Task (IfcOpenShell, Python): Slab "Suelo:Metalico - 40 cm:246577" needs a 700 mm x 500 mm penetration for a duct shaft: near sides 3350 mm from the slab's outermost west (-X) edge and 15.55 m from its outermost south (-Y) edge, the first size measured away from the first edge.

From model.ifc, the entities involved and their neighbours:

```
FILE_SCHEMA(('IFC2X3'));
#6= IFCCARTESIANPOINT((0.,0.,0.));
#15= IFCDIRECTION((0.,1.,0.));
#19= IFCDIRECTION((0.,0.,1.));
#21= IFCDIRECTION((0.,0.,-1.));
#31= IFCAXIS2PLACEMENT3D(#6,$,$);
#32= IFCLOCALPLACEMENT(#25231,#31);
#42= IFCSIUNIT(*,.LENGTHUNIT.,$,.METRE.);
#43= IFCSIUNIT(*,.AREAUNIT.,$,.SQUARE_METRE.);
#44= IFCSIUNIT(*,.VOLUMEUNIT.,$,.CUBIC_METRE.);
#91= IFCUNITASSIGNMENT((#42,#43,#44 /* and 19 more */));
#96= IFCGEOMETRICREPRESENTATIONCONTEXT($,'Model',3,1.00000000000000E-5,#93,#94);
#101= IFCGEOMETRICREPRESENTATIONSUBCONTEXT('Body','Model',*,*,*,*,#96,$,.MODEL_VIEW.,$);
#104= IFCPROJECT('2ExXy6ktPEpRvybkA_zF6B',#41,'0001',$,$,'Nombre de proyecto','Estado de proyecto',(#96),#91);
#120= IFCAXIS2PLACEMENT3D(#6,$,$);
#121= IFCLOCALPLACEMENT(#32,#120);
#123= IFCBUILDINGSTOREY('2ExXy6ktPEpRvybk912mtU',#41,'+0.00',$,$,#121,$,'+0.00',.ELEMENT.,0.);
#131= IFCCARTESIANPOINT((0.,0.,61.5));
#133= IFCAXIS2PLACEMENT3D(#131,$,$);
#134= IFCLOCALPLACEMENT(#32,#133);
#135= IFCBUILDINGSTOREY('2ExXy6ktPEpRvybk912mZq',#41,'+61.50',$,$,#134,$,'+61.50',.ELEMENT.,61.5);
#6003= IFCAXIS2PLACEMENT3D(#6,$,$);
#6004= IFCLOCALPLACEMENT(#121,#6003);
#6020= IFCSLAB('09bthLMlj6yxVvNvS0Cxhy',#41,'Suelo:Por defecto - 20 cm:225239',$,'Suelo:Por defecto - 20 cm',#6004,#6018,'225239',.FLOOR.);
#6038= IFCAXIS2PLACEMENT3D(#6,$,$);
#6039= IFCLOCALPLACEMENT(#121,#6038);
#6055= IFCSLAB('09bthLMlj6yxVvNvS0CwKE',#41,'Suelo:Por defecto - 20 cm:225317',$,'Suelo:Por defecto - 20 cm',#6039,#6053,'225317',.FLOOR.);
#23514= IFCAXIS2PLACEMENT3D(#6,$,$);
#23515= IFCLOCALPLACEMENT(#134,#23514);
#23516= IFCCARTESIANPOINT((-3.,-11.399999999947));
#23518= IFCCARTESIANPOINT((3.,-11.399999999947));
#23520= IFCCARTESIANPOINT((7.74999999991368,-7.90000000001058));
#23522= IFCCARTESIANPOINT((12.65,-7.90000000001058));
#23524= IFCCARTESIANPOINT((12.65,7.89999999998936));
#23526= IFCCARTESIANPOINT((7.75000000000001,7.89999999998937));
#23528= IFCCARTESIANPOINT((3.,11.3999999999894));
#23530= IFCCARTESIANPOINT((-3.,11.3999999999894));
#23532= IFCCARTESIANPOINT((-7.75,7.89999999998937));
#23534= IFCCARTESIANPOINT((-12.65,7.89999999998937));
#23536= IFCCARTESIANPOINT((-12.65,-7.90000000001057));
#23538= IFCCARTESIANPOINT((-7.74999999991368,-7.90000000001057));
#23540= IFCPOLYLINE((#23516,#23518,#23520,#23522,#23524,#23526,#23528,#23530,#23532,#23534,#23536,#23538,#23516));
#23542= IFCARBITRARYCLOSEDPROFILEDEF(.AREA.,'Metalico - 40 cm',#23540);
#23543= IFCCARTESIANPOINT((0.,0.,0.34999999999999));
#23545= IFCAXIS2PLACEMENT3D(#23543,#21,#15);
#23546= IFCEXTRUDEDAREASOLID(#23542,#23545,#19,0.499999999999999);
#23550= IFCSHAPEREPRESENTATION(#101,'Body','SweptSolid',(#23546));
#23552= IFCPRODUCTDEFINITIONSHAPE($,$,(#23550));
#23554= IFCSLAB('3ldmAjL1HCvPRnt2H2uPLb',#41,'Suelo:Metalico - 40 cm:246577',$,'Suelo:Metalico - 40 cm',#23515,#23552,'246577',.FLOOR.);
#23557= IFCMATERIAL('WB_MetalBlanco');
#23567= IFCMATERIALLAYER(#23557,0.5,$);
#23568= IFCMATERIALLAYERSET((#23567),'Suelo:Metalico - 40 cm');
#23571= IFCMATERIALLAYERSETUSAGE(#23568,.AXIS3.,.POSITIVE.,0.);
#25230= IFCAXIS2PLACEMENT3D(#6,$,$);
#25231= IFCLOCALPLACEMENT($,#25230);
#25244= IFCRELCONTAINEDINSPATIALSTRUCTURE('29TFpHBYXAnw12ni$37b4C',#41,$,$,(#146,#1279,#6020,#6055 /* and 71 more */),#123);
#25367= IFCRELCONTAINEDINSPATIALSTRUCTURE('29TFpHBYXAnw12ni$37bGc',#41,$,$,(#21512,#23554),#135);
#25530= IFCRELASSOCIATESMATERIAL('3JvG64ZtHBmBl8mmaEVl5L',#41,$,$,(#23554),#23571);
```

```python
import numpy as np
import ifcopenshell
import ifcopenshell.api.feature
import ifcopenshell.api.geometry
import ifcopenshell.api.root
import ifcopenshell.geom
import ifcopenshell.util.placement
import ifcopenshell.util.representation
import ifcopenshell.util.shape
import ifcopenshell.util.unit

model = ifcopenshell.open("model.ifc")
unit_scale = ifcopenshell.util.unit.calculate_unit_scale(model)
settings = ifcopenshell.geom.settings()


def volume(element):
    """Net volume in cubic metres, openings subtracted."""
    shape = ifcopenshell.geom.create_shape(settings, element)
    return ifcopenshell.util.shape.get_volume(shape.geometry)


slab = model.by_guid("3ldmAjL1HCvPRnt2H2uPLb")
before = volume(slab)

# Extent in the slab's own axes, in metres. The edges named are its -X and -Y sides.
slab_shape = ifcopenshell.geom.create_shape(settings, slab)
vertices = ifcopenshell.util.shape.get_vertices(slab_shape.geometry)
x_min, y_min, bottom = vertices.min(axis=0)
top = vertices[:, 2].max()

opening = ifcopenshell.api.root.create_entity(model, ifc_class="IfcOpeningElement", name="Duct shaft opening")
context = ifcopenshell.util.representation.get_context(model, "Model", "Body", "MODEL_VIEW")
width, depth = 0.7, 0.5
outline = [(0.0, 0.0), (width, 0.0), (width, depth), (0.0, depth), (0.0, 0.0)]
# Overshoot both faces by 50 mm so the cut is clean.
shape = ifcopenshell.api.geometry.add_slab_representation(
    model, context=context, depth=top - bottom + 0.1, polyline=outline
)
ifcopenshell.api.geometry.assign_representation(model, product=opening, representation=shape)

matrix = ifcopenshell.util.placement.get_local_placement(slab.ObjectPlacement)
matrix[:, 3] = matrix @ np.append(np.array([x_min + 3.35, y_min + 15.55, bottom - 0.05]) / unit_scale, 1.0)
ifcopenshell.api.geometry.edit_object_placement(model, product=opening, matrix=matrix, is_si=False)
ifcopenshell.api.feature.add_feature(model, feature=opening, element=slab)

after = volume(slab)

print(f"slab volume {before:.3f} -> {after:.3f} m3")

model.write("model-out.ifc")
```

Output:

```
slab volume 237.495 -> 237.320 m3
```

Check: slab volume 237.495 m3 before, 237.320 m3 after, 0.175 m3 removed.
